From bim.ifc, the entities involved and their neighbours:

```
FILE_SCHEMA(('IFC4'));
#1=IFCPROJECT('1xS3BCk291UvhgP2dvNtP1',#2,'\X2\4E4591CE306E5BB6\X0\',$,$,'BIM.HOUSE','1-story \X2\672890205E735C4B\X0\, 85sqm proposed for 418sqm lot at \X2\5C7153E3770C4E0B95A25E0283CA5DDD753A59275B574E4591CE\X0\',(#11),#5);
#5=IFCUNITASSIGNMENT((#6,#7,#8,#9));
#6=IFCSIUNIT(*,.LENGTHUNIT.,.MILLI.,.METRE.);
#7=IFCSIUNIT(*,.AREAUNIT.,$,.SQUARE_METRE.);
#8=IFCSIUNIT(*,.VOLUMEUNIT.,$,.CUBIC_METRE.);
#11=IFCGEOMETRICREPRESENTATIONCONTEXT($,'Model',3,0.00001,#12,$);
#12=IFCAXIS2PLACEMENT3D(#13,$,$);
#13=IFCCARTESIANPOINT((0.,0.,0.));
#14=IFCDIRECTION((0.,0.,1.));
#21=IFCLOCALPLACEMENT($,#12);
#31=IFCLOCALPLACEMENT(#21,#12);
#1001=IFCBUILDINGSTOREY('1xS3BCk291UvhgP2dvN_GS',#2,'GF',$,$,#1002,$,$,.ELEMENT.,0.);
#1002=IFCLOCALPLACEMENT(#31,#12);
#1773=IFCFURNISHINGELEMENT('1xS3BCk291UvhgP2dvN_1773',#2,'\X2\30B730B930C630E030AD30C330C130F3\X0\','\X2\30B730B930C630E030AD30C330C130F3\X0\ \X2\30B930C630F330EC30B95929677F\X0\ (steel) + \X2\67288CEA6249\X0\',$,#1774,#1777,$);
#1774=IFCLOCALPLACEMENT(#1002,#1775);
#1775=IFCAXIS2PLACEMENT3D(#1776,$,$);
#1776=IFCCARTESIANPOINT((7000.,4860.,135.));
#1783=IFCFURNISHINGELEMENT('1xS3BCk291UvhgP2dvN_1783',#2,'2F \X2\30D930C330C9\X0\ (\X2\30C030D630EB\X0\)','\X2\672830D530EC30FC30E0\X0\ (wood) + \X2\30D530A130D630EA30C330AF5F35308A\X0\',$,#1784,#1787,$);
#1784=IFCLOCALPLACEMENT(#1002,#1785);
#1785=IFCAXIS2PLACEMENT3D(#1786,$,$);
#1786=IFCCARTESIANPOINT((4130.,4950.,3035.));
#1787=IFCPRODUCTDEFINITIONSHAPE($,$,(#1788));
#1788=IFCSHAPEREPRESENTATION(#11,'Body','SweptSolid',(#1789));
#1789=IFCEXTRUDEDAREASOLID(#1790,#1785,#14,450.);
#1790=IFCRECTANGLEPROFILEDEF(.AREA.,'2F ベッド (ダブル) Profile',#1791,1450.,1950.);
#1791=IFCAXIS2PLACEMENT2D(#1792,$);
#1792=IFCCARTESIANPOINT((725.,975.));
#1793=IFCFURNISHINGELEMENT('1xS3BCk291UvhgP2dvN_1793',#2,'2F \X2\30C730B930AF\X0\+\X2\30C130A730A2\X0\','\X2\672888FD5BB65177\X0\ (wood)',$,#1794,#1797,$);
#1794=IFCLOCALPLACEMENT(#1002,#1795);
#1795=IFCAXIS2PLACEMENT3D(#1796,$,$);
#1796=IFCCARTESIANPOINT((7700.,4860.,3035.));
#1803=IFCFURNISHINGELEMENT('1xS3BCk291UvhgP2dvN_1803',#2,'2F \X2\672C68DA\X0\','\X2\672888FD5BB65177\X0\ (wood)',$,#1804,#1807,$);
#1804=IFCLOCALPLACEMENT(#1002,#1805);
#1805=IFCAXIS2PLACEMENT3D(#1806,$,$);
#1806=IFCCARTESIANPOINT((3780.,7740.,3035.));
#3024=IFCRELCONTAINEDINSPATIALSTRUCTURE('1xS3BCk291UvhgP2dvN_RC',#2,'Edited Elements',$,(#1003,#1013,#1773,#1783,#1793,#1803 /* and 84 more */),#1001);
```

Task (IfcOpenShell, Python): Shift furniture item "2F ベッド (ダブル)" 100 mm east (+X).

```python
import ifcopenshell
import ifcopenshell.api.geometry
import ifcopenshell.util.placement

model = ifcopenshell.open("bim.ifc")

item = model.by_id(1783)
matrix = ifcopenshell.util.placement.get_local_placement(item.ObjectPlacement)
matrix[0, 3] += 100.0
ifcopenshell.api.geometry.edit_object_placement(model, product=item, matrix=matrix, is_si=False)

print(ifcopenshell.util.placement.get_local_placement(item.ObjectPlacement).round(3) + 0.0)

model.write("bim_v2.ifc")
```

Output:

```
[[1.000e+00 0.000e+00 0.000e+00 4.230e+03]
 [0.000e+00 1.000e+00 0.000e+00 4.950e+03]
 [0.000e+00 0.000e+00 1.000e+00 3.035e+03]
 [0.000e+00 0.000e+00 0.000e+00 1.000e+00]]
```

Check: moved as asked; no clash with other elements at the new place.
